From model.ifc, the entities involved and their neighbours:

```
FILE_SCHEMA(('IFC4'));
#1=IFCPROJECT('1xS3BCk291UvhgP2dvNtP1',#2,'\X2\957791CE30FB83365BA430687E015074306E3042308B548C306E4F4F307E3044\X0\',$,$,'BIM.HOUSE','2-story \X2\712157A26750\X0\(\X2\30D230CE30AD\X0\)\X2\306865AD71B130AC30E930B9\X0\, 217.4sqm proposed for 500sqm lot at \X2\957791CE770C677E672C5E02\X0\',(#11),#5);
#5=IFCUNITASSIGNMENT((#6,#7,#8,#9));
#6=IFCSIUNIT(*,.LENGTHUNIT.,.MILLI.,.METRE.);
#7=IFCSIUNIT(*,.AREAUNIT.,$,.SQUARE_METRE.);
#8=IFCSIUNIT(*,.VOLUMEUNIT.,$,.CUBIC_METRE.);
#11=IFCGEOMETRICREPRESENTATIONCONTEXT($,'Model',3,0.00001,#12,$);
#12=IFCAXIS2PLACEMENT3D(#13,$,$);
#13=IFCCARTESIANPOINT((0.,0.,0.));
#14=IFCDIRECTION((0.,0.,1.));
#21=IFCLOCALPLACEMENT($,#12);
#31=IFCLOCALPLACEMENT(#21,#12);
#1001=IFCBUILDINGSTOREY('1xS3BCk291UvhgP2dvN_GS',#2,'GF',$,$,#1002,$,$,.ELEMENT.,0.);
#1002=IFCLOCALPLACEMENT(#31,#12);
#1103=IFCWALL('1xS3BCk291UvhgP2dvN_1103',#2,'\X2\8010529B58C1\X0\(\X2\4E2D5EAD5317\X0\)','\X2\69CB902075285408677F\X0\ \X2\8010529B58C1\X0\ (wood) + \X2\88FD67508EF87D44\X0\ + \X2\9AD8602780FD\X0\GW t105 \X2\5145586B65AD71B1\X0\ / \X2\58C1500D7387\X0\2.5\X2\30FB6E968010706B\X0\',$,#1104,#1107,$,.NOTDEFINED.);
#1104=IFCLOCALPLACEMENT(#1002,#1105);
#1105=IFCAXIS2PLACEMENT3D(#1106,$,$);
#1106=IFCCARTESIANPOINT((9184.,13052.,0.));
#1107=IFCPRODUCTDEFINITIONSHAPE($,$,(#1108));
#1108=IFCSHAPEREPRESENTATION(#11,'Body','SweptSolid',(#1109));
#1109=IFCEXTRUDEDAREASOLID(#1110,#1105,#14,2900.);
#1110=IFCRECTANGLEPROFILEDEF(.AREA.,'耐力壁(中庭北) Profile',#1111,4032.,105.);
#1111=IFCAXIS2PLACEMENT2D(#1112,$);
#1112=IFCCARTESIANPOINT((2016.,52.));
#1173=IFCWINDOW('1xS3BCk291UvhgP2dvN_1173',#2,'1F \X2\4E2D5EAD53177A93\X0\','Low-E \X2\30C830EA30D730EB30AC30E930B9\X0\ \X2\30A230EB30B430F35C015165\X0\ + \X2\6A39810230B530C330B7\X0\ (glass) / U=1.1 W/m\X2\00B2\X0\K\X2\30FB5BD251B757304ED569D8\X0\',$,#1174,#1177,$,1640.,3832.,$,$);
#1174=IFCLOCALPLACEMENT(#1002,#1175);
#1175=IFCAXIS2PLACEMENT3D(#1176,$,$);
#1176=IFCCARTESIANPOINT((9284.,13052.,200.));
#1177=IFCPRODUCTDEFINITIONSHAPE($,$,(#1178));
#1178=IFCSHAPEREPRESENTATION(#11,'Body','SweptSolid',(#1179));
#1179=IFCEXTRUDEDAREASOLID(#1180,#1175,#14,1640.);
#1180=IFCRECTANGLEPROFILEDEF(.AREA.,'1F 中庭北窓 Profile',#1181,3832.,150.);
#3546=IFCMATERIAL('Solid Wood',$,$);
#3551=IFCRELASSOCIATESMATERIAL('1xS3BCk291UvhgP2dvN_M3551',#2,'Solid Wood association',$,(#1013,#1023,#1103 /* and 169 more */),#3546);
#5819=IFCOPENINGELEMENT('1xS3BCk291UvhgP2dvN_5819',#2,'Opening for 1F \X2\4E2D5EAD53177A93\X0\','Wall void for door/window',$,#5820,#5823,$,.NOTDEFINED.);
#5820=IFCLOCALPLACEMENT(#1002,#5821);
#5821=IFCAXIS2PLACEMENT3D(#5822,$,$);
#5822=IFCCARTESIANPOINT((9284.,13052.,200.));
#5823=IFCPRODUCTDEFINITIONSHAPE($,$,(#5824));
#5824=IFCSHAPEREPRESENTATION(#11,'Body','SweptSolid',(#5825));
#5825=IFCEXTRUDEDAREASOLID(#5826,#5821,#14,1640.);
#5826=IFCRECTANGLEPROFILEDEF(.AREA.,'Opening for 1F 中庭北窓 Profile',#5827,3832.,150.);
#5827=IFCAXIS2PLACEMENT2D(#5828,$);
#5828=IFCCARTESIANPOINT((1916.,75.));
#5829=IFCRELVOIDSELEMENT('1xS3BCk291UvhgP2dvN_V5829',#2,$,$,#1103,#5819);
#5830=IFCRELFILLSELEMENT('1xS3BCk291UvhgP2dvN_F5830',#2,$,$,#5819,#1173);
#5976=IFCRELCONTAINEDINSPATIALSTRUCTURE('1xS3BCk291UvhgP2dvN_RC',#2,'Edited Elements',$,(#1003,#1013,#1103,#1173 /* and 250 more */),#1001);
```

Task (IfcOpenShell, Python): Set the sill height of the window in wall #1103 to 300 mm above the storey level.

```python
import numpy as np
import ifcopenshell
import ifcopenshell.api.geometry
import ifcopenshell.geom
import ifcopenshell.util.element
import ifcopenshell.util.placement
import ifcopenshell.util.shape
import ifcopenshell.util.unit

model = ifcopenshell.open("model.ifc")
unit_scale = ifcopenshell.util.unit.calculate_unit_scale(model)

window = model.by_guid("1xS3BCk291UvhgP2dvN_1173")
opening = window.FillsVoids[0].RelatingOpeningElement
storey = ifcopenshell.util.element.get_container(window, ifc_class="IfcBuildingStorey")
level = ifcopenshell.util.placement.get_local_placement(storey.ObjectPlacement)[2, 3]

# The opening's origin need not be at the sill, so measure its lowest point.
shape = ifcopenshell.geom.create_shape(ifcopenshell.geom.settings(), opening)
bottom = ifcopenshell.util.shape.get_shape_bottom_elevation(shape, shape.geometry) / unit_scale
dz = level + 300.0 - bottom

shift = np.array([0.0, 0.0, dz])
# The window is not placed relative to its opening, so move both.
for product in (opening, window):
    matrix = ifcopenshell.util.placement.get_local_placement(product.ObjectPlacement)
    matrix[:3, 3] += shift
    ifcopenshell.api.geometry.edit_object_placement(model, product=product, matrix=matrix, is_si=False)

print(f"moved by {dz * unit_scale:+.3f} m")

model.write("model_v2.ifc")
```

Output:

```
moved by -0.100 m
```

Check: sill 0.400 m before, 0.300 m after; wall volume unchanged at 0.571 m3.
